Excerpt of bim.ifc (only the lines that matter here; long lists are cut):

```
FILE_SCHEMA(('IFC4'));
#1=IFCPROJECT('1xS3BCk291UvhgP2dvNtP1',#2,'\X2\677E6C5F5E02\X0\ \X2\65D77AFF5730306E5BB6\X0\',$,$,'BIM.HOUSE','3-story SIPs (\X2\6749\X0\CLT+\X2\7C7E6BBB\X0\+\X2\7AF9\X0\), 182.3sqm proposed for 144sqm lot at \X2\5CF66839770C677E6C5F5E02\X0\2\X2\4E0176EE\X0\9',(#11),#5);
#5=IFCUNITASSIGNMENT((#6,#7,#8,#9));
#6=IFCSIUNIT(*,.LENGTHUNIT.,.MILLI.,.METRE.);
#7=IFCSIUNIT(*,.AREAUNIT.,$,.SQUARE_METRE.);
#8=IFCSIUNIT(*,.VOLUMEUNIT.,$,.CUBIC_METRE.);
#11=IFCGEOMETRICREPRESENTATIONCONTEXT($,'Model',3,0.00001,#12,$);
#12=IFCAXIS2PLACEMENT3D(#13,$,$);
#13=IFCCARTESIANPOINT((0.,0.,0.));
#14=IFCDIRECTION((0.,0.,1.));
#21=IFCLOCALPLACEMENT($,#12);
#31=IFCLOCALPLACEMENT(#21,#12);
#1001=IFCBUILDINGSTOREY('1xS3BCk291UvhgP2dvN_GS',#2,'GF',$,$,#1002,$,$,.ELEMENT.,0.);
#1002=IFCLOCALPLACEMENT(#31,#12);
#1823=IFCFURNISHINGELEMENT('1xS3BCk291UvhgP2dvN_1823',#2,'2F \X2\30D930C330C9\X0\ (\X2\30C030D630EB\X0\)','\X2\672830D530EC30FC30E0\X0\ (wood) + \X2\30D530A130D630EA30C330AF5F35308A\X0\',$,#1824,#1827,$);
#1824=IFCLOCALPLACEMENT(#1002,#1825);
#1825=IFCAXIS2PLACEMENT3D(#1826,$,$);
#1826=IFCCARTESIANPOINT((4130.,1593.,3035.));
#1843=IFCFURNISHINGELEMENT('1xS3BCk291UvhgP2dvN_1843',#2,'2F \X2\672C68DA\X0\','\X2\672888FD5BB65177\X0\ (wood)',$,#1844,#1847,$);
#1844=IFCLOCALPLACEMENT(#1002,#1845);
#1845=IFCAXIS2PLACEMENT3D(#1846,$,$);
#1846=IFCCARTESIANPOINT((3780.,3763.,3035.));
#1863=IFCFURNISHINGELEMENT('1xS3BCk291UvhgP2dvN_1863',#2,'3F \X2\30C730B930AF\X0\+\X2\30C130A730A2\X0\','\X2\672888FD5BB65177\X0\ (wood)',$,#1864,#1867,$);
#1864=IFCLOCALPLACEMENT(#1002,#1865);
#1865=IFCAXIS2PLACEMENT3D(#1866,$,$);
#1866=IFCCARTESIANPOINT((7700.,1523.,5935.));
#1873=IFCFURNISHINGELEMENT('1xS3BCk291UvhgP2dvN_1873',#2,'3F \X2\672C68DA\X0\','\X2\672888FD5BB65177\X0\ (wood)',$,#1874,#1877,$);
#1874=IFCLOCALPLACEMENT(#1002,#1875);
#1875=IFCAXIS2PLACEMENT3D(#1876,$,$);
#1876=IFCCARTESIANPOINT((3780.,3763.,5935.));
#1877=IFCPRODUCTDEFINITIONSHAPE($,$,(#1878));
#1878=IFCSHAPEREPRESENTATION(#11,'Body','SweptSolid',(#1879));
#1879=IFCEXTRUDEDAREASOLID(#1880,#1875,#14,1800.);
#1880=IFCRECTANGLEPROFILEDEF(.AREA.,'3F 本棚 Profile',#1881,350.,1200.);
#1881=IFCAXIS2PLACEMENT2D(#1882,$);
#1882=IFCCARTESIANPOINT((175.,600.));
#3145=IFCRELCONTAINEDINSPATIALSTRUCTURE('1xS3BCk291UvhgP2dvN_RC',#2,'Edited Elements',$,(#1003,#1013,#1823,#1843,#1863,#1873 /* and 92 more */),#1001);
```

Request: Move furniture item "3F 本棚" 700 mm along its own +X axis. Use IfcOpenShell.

```python
import ifcopenshell
import ifcopenshell.api.geometry
import ifcopenshell.util.placement

model = ifcopenshell.open("bim.ifc")

item = model.by_guid("1xS3BCk291UvhgP2dvN_1873")
matrix = ifcopenshell.util.placement.get_local_placement(item.ObjectPlacement)
matrix[:3, 3] += matrix[:3, 0] * 700.0
ifcopenshell.api.geometry.edit_object_placement(model, product=item, matrix=matrix, is_si=False)

print(ifcopenshell.util.placement.get_local_placement(item.ObjectPlacement).round(3) + 0.0)

model.write("bim_rev.ifc")
```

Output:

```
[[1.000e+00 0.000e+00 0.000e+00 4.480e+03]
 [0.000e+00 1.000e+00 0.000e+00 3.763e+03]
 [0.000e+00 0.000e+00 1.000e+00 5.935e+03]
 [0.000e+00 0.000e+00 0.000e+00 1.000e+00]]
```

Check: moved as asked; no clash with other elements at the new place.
